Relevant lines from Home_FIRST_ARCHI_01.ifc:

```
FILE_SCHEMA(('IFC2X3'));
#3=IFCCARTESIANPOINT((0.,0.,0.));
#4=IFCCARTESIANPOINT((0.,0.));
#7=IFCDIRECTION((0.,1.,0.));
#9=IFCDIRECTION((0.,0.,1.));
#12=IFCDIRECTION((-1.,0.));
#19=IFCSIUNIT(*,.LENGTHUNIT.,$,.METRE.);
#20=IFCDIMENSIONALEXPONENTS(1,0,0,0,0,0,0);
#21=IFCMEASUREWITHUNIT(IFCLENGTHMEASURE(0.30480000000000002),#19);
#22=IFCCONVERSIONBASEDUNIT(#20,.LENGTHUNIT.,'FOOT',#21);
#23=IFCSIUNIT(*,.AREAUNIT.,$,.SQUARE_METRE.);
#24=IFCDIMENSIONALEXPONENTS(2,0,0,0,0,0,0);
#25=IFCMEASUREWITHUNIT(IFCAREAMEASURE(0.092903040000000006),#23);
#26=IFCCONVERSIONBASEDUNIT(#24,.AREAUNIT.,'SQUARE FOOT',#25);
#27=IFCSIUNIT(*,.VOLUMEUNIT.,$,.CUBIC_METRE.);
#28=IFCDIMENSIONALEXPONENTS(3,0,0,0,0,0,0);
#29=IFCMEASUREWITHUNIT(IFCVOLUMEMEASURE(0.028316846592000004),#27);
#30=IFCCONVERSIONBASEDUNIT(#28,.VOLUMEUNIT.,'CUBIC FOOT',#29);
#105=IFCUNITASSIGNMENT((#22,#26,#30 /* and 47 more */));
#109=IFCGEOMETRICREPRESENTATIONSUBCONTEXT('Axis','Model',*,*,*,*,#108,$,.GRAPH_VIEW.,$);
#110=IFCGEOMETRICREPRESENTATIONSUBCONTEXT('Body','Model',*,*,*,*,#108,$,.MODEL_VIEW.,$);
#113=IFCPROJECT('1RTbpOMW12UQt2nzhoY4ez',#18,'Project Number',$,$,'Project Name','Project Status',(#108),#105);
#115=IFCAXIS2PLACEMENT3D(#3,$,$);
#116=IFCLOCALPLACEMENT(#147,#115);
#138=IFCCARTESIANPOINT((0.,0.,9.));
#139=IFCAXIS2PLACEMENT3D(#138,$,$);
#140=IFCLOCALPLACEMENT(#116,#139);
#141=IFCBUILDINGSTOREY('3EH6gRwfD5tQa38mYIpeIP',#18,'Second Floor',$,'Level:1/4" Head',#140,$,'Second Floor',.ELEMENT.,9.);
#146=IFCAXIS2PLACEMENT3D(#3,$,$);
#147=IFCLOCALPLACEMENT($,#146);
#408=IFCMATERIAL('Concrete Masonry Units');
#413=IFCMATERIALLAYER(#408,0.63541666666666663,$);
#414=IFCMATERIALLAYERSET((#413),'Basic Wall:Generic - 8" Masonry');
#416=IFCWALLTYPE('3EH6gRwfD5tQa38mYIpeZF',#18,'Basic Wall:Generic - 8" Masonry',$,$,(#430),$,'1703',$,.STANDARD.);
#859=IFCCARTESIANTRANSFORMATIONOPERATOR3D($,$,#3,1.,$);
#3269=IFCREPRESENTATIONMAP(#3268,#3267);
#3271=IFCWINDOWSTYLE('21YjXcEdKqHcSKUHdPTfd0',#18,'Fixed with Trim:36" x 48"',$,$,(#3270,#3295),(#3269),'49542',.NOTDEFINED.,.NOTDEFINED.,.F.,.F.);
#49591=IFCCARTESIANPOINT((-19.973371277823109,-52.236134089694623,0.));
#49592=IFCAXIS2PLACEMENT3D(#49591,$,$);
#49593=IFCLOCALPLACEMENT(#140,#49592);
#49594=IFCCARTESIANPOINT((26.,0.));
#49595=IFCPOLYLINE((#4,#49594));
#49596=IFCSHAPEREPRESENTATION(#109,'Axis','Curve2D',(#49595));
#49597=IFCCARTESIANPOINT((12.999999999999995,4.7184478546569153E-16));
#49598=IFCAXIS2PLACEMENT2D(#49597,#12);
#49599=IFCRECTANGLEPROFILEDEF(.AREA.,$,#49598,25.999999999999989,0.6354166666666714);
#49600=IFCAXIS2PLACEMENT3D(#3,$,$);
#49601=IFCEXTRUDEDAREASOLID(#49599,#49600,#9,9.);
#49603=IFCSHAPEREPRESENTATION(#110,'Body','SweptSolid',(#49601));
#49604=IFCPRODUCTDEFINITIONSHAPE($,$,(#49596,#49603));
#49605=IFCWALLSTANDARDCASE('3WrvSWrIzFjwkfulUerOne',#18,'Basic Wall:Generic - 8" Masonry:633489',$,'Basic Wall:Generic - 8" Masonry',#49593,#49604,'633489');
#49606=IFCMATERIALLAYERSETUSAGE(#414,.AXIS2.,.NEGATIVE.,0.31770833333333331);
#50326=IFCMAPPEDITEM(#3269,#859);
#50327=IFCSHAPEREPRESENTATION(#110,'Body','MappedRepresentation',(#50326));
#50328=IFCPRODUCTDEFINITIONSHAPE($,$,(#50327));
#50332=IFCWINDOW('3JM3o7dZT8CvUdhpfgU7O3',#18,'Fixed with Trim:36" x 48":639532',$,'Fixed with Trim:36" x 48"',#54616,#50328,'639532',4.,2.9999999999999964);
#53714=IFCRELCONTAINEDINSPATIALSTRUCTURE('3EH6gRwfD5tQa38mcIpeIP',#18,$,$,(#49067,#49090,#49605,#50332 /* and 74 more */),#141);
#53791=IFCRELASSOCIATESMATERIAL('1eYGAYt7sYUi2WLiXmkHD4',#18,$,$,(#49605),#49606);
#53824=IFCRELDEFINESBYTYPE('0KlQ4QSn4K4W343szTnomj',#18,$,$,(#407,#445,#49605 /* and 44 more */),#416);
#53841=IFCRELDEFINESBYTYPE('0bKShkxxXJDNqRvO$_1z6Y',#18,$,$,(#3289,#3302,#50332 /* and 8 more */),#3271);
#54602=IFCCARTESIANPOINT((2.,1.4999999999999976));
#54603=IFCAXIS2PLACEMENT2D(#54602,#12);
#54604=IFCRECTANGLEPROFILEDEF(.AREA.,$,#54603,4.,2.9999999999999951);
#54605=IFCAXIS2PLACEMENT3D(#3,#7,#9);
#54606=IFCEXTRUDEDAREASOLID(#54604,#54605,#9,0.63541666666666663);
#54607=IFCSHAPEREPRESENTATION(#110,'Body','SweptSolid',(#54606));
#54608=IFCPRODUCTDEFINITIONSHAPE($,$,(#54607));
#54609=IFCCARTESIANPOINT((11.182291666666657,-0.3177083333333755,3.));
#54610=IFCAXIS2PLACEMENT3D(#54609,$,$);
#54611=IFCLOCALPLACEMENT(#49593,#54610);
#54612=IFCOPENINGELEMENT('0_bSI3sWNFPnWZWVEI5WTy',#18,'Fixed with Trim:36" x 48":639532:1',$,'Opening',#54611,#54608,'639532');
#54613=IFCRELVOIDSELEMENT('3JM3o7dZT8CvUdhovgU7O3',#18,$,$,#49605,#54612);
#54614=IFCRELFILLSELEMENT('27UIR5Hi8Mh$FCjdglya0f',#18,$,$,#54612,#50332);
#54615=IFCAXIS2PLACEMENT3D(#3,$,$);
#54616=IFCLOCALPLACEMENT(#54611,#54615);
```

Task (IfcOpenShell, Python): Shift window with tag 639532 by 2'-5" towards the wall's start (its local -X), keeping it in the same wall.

```python
import ifcopenshell
import ifcopenshell.api.geometry
import ifcopenshell.util.placement
import ifcopenshell.util.unit

model = ifcopenshell.open("Home_FIRST_ARCHI_01.ifc")
unit_scale = ifcopenshell.util.unit.calculate_unit_scale(model)

window = model.by_guid("3JM3o7dZT8CvUdhpfgU7O3")
opening = window.FillsVoids[0].RelatingOpeningElement
wall = opening.VoidsElements[0].RelatingBuildingElement

wall_matrix = ifcopenshell.util.placement.get_local_placement(wall.ObjectPlacement)
shift = wall_matrix[:3, 0] * -29 * 0.0254 / unit_scale
before = ifcopenshell.util.placement.get_local_placement(window.ObjectPlacement)[:3, 3].copy()

# The window is placed relative to its opening, so it follows when the opening moves.
matrix = ifcopenshell.util.placement.get_local_placement(opening.ObjectPlacement)
matrix[:3, 3] += shift
ifcopenshell.api.geometry.edit_object_placement(
    model, product=opening, matrix=matrix, is_si=False, should_transform_children=True
)

after = ifcopenshell.util.placement.get_local_placement(window.ObjectPlacement)[:3, 3]
print("window moved by", (after - before).round(3) + 0.0)

model.write("Home_FIRST_ARCHI_01_rev.ifc")
```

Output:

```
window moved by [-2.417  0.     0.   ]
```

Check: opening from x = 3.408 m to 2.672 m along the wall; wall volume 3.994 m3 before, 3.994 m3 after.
